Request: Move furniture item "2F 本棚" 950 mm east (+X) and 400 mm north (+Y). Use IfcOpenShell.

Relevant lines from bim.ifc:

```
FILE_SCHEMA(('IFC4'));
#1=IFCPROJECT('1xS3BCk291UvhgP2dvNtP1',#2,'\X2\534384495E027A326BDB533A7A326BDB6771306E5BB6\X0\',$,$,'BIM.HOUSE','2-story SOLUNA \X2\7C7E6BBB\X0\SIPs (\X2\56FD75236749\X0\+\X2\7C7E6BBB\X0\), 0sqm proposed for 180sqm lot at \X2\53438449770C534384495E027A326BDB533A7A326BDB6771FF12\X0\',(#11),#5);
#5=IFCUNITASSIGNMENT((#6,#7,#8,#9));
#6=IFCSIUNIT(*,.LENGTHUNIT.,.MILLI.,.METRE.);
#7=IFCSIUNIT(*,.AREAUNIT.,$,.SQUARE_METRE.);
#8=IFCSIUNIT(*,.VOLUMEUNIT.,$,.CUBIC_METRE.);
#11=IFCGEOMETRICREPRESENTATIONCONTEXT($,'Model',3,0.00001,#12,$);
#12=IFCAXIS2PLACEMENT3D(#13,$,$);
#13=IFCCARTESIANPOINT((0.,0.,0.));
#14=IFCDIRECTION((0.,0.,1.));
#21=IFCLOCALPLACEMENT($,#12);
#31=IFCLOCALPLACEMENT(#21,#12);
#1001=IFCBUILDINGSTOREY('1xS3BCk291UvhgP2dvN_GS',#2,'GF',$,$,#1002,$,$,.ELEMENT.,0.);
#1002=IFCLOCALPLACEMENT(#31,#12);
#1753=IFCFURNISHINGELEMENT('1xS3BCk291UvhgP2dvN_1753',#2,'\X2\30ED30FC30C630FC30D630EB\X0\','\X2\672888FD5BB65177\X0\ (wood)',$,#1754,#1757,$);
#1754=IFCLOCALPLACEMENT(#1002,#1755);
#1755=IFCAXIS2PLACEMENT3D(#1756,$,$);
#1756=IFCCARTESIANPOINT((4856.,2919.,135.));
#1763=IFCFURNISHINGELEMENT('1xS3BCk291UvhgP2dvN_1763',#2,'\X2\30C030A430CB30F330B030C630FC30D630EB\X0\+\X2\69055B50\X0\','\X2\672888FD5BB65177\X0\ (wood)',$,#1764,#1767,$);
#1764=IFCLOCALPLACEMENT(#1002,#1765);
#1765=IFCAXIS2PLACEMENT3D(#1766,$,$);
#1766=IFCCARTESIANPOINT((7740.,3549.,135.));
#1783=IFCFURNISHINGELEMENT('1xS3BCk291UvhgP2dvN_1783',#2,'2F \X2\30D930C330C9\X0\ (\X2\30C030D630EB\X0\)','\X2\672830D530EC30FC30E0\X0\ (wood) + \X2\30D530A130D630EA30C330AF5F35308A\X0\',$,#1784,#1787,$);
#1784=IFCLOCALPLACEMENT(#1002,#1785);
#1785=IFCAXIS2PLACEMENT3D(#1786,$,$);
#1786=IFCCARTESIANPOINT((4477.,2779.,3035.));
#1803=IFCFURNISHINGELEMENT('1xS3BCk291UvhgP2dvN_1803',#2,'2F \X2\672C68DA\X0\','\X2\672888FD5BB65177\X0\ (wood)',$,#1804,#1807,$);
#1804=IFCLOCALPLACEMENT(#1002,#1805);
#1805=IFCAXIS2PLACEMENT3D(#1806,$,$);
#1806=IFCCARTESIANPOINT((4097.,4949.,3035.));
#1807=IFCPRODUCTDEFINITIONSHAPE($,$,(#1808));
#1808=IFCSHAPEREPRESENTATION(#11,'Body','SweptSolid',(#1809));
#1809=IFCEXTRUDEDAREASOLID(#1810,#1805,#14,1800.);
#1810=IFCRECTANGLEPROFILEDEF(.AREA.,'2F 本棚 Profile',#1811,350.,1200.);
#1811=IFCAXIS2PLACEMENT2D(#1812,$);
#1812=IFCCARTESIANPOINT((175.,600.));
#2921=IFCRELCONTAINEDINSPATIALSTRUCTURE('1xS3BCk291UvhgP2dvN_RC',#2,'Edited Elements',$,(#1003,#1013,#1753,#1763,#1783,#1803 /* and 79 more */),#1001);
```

```python
import ifcopenshell
import ifcopenshell.api.geometry
import ifcopenshell.util.placement
import ifcopenshell.util.unit

model = ifcopenshell.open("bim.ifc")
unit_scale = ifcopenshell.util.unit.calculate_unit_scale(model)

item = model.by_guid("1xS3BCk291UvhgP2dvN_1803")
matrix = ifcopenshell.util.placement.get_local_placement(item.ObjectPlacement)
matrix[0, 3] += 0.95 / unit_scale
matrix[1, 3] += 0.4 / unit_scale
ifcopenshell.api.geometry.edit_object_placement(model, product=item, matrix=matrix, is_si=False)

print(ifcopenshell.util.placement.get_local_placement(item.ObjectPlacement).round(3) + 0.0)

model.write("bim_v2.ifc")
```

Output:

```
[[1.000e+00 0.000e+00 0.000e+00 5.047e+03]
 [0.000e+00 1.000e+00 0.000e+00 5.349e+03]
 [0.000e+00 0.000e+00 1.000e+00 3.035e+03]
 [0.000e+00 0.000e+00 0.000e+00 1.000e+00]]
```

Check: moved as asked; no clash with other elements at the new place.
